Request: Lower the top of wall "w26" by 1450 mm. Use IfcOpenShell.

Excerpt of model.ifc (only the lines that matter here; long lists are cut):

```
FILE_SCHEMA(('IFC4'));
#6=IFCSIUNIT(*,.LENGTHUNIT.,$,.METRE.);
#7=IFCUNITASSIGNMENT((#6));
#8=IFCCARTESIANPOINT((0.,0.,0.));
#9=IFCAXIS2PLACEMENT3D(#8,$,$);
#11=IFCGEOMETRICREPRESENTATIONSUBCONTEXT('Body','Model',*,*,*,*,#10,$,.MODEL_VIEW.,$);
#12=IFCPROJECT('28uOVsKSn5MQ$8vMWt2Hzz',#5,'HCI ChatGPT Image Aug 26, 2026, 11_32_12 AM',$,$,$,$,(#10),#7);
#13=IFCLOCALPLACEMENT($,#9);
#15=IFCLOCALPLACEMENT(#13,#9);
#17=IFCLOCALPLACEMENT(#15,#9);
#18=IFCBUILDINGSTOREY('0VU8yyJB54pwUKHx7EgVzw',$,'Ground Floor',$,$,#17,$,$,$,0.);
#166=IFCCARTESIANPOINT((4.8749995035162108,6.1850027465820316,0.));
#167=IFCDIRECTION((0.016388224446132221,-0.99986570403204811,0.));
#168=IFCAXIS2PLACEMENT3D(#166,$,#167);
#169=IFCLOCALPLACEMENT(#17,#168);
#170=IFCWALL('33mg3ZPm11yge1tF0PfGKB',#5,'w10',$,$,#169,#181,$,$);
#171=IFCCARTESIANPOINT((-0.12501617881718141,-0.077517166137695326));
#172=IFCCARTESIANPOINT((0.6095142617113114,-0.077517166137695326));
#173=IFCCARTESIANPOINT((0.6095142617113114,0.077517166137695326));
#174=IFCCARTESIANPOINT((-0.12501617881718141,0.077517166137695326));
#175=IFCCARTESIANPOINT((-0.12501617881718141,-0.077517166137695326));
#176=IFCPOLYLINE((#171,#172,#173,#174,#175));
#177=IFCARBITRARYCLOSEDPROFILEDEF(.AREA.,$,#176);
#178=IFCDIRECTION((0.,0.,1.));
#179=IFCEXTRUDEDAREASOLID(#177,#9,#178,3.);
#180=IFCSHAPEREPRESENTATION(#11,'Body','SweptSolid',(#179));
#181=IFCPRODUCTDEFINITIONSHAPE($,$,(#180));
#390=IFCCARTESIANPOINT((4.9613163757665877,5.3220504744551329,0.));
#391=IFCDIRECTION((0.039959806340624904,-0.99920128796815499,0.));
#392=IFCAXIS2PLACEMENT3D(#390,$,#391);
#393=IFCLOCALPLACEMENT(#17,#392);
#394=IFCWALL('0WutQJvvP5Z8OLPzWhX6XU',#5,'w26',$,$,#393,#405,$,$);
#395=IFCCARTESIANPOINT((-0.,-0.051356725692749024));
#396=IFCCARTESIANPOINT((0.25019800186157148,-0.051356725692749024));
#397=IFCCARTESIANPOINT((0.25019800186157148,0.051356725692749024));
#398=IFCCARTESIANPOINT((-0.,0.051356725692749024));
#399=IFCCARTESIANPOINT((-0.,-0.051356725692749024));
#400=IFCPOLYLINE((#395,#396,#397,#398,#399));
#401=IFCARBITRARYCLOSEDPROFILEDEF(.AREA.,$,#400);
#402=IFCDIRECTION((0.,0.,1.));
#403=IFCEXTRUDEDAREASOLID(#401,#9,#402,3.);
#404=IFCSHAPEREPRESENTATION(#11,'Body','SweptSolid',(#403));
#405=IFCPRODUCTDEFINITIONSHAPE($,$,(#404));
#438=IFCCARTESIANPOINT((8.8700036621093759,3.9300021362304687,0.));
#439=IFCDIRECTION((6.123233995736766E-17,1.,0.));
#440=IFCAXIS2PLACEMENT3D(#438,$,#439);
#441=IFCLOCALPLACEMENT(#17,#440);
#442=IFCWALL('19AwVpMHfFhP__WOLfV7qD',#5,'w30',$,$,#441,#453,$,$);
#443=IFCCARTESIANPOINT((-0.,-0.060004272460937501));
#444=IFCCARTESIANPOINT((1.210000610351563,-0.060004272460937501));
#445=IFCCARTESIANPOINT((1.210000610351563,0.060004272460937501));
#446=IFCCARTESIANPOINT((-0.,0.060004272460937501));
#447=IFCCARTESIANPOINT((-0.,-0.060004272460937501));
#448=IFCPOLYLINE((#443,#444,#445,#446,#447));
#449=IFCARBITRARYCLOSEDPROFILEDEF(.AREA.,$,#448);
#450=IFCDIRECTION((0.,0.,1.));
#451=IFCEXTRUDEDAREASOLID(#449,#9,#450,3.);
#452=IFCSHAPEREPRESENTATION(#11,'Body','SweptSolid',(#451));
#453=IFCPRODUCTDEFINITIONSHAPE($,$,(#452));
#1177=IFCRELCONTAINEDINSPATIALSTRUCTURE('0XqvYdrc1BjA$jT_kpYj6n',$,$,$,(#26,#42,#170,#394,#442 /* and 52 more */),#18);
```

```python
import ifcopenshell
import ifcopenshell.geom
import ifcopenshell.util.representation
import ifcopenshell.util.shape
import ifcopenshell.util.unit

model = ifcopenshell.open("model.ifc")
unit_scale = ifcopenshell.util.unit.calculate_unit_scale(model)
settings = ifcopenshell.geom.settings()


def volume(element):
    """Net volume in cubic metres, openings subtracted."""
    shape = ifcopenshell.geom.create_shape(settings, element)
    return ifcopenshell.util.shape.get_volume(shape.geometry)


wall = model.by_guid("0WutQJvvP5Z8OLPzWhX6XU")
before = volume(wall)

body = ifcopenshell.util.representation.get_representation(wall, "Model", "Body")
solid = body.Items[0]
old_height = solid.Depth
solid.Depth -= 1.45 / unit_scale
after = volume(wall)

print(f"height {old_height:g} -> {solid.Depth:g}, volume {before:.3f} -> {after:.3f} m3")

model.write("model_rev.ifc")
```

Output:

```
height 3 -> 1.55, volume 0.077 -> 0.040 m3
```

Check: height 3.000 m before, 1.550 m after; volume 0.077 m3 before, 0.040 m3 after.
